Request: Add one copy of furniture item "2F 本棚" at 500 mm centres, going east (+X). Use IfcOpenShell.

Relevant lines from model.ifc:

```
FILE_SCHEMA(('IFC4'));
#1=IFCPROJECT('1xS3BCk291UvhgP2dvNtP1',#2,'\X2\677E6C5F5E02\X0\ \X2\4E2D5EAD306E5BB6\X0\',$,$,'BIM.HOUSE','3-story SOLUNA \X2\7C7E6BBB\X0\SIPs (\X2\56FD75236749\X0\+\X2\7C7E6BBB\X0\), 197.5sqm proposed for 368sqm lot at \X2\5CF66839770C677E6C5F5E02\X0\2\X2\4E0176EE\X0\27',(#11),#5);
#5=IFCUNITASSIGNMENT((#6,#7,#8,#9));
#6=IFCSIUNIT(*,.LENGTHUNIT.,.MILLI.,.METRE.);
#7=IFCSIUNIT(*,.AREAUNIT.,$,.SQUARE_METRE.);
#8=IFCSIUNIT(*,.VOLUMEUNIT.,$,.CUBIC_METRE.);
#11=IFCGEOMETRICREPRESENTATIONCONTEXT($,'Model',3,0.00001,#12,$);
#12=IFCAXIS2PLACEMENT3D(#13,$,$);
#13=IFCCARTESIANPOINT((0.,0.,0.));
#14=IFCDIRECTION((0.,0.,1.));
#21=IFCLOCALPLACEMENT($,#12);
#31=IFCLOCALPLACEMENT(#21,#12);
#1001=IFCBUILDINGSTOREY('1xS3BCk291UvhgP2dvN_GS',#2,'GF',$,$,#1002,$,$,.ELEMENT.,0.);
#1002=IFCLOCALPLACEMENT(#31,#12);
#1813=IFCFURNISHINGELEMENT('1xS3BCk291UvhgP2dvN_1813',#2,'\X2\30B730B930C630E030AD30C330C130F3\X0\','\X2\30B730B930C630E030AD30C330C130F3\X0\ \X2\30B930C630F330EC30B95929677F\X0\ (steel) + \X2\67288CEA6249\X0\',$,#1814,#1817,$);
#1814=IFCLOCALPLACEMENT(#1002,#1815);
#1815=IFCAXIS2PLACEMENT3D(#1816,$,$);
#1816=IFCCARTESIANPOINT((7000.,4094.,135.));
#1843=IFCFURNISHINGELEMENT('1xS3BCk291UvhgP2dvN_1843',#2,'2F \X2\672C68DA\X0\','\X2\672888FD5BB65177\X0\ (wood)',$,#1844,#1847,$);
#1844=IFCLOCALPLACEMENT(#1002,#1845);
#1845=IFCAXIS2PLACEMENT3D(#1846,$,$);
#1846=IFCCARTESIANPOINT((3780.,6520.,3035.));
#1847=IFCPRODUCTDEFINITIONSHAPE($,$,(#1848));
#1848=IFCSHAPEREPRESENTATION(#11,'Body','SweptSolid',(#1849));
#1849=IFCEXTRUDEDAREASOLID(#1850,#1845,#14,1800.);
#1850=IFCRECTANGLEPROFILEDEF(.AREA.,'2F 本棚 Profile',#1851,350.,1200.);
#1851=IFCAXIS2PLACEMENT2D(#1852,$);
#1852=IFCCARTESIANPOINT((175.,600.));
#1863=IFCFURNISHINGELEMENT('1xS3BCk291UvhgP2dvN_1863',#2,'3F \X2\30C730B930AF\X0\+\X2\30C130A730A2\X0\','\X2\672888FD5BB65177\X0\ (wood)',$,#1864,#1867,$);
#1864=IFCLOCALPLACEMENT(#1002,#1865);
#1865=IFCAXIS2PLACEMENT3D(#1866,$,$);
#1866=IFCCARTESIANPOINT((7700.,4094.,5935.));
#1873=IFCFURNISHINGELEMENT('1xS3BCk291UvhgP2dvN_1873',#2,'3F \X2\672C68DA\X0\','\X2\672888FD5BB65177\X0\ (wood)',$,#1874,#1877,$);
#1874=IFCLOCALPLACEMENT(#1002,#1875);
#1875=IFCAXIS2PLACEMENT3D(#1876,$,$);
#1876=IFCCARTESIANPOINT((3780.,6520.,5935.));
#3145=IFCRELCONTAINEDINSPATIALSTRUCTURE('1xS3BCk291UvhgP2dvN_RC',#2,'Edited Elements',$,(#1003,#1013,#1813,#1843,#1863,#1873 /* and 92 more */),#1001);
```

```python
import numpy as np
import ifcopenshell
import ifcopenshell.api.geometry
import ifcopenshell.api.root
import ifcopenshell.util.element
import ifcopenshell.util.placement

model = ifcopenshell.open("model.ifc")


def reuse_history(source, copy):
    """copy_class also copies each property set's owner history, people and application; keep the originals."""
    for rel in copy.IsDefinedBy:
        if rel.is_a("IfcRelDefinesByProperties") and (history := rel.RelatingPropertyDefinition.OwnerHistory):
            rel.RelatingPropertyDefinition.OwnerHistory = source.OwnerHistory
            ifcopenshell.util.element.remove_deep2(model, history)


source = model.by_id(1843)
base = ifcopenshell.util.placement.get_local_placement(source.ObjectPlacement)
step = np.array([1.0, 0.0, 0.0]) * 500.0

for i in range(1, 2):
    copy = ifcopenshell.api.root.copy_class(model, product=source)
    copy.Representation = ifcopenshell.util.element.copy_deep(
        model, source.Representation, exclude=["IfcGeometricRepresentationContext", "IfcRepresentationMap"]
    )
    reuse_history(source, copy)
    matrix = base.copy()
    matrix[:3, 3] += i * step
    print("added at", matrix[:3, 3].round(3) + 0.0)
    ifcopenshell.api.geometry.edit_object_placement(model, product=copy, matrix=matrix, is_si=False)

model.write("model_v2.ifc")
```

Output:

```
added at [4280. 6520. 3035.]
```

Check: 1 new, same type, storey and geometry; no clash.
